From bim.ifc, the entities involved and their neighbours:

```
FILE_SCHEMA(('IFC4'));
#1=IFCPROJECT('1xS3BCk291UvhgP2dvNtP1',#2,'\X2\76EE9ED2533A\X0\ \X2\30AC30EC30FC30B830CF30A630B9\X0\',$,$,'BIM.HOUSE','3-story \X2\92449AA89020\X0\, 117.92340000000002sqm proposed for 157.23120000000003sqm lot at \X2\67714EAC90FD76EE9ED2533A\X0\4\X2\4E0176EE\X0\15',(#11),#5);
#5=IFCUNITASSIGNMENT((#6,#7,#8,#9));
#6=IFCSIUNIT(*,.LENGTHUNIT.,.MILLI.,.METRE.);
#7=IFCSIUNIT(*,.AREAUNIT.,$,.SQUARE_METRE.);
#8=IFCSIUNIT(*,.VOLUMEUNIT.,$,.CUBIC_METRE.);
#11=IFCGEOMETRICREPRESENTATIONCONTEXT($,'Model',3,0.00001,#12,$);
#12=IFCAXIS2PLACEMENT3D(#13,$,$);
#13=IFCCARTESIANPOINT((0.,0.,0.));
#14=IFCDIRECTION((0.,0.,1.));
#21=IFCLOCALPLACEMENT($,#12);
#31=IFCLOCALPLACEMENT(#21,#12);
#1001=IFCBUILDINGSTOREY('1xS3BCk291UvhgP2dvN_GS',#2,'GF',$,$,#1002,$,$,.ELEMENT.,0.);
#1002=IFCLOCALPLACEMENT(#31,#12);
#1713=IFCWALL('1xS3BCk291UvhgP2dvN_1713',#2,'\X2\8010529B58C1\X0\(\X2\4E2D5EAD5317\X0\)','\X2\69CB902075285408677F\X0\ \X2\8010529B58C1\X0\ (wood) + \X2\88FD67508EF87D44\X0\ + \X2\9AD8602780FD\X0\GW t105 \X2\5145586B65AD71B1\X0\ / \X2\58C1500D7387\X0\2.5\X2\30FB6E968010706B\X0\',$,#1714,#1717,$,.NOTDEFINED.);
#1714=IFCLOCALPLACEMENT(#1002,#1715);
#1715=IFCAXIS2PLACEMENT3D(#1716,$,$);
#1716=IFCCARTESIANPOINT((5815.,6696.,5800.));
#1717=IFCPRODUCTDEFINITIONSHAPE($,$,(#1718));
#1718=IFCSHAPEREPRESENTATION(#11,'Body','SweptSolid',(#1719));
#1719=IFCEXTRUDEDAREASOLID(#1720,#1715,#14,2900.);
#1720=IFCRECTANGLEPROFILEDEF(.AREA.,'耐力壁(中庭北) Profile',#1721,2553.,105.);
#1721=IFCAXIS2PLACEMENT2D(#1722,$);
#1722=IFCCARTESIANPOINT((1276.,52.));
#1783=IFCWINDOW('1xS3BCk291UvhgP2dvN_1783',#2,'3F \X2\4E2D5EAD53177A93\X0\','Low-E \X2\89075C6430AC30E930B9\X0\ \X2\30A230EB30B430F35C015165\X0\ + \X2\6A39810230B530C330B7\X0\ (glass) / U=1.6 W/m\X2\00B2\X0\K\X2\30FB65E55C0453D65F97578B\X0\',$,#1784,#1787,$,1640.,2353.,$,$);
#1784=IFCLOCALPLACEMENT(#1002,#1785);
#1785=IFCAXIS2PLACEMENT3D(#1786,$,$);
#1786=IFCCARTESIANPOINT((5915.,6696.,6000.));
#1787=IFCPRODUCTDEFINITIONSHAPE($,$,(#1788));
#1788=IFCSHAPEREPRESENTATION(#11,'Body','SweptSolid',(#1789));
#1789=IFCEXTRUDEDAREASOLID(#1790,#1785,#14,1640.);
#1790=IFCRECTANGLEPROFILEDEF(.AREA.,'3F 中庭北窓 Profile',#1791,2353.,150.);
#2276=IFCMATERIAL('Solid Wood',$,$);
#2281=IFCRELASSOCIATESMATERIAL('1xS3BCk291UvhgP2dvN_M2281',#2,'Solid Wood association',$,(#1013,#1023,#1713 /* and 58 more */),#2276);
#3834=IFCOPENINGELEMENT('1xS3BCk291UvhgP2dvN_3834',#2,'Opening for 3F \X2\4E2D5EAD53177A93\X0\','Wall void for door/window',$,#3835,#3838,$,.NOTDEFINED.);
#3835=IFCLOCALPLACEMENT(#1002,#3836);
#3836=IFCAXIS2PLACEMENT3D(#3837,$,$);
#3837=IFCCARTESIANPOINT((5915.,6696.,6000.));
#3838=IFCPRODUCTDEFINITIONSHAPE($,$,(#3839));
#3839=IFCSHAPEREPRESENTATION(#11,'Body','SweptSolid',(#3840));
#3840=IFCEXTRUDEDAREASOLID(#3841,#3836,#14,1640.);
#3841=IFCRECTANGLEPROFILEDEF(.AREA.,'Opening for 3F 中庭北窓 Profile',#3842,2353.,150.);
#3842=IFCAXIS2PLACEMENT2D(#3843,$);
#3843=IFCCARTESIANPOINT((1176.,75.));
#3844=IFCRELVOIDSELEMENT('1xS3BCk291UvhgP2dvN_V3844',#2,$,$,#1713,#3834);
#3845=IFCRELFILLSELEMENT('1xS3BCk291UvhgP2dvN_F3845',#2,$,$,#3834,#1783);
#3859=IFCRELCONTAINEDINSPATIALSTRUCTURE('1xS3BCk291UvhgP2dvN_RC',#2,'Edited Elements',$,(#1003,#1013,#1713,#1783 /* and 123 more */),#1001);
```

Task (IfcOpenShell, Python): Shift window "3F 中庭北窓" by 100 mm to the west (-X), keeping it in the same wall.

```python
import ifcopenshell
import ifcopenshell.api.geometry
import ifcopenshell.util.placement
import ifcopenshell.util.unit

model = ifcopenshell.open("bim.ifc")
unit_scale = ifcopenshell.util.unit.calculate_unit_scale(model)

window = model.by_guid("1xS3BCk291UvhgP2dvN_1783")
opening = window.FillsVoids[0].RelatingOpeningElement
wall = opening.VoidsElements[0].RelatingBuildingElement

wall_matrix = ifcopenshell.util.placement.get_local_placement(wall.ObjectPlacement)
shift = wall_matrix[:3, 0] * -0.1 / unit_scale
before = ifcopenshell.util.placement.get_local_placement(window.ObjectPlacement)[:3, 3].copy()

# The window is not placed relative to its opening, so move both.
for product in (opening, window):
    matrix = ifcopenshell.util.placement.get_local_placement(product.ObjectPlacement)
    matrix[:3, 3] += shift
    ifcopenshell.api.geometry.edit_object_placement(model, product=product, matrix=matrix, is_si=False)

after = ifcopenshell.util.placement.get_local_placement(window.ObjectPlacement)[:3, 3]
print("window moved by", (after - before).round(3) + 0.0)

model.write("bim_rev.ifc")
```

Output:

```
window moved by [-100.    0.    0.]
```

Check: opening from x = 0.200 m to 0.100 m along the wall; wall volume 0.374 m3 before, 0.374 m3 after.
